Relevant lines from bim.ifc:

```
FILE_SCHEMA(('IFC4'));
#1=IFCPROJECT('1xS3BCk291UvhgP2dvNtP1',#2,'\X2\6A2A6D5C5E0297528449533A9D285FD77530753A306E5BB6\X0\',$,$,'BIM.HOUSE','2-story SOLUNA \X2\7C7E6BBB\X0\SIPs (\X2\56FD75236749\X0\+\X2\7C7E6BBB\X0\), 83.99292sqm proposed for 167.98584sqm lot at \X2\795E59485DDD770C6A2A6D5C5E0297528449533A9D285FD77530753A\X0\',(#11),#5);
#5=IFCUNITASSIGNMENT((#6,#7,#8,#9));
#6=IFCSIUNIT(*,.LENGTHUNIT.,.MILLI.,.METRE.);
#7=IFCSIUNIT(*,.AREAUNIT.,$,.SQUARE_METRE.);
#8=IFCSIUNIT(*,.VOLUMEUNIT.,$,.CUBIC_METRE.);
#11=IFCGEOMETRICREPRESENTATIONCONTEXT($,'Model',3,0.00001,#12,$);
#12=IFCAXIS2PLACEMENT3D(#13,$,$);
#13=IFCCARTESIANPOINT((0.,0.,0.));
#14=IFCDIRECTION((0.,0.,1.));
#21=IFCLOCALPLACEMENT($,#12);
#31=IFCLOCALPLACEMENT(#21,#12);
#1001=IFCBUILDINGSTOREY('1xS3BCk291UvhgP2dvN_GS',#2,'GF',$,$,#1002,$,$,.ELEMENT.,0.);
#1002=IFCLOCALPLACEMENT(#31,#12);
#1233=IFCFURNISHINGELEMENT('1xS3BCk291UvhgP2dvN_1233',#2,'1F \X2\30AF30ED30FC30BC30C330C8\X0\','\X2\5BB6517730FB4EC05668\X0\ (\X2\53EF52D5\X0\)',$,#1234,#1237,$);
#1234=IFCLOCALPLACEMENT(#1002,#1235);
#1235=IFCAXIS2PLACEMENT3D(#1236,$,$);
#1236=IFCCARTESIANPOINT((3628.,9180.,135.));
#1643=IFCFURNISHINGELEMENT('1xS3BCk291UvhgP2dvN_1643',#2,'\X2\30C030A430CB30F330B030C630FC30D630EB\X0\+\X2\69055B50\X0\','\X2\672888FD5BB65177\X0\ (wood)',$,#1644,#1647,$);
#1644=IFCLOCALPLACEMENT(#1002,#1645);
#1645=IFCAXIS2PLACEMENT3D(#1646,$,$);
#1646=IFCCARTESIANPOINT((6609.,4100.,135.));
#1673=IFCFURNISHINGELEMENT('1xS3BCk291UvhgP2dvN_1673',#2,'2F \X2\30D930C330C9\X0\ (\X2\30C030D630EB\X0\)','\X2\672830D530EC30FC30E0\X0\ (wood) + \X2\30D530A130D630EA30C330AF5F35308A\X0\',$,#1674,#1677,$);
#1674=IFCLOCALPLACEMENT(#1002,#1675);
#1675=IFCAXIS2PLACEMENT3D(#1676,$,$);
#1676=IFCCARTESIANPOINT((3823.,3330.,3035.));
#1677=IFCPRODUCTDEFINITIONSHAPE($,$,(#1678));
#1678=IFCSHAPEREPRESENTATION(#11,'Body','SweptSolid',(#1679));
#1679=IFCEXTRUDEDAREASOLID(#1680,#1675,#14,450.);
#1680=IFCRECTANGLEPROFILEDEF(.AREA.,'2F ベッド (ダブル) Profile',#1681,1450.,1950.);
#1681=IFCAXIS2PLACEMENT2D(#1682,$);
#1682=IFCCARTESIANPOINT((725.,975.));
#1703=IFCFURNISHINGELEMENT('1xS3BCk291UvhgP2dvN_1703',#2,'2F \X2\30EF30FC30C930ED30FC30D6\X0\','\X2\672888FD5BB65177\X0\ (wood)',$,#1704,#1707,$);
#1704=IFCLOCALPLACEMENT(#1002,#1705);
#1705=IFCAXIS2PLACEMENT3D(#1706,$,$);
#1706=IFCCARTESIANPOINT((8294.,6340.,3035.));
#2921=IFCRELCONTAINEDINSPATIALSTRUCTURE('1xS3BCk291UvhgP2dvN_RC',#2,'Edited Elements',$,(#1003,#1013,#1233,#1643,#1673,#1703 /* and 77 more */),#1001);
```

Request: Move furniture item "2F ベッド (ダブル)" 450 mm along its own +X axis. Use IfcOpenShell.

```python
import ifcopenshell
import ifcopenshell.api.geometry
import ifcopenshell.util.placement
import ifcopenshell.util.unit

model = ifcopenshell.open("bim.ifc")
unit_scale = ifcopenshell.util.unit.calculate_unit_scale(model)

item = model.by_id(1673)
matrix = ifcopenshell.util.placement.get_local_placement(item.ObjectPlacement)
matrix[:3, 3] += matrix[:3, 0] * 0.45 / unit_scale
ifcopenshell.api.geometry.edit_object_placement(model, product=item, matrix=matrix, is_si=False)

print(ifcopenshell.util.placement.get_local_placement(item.ObjectPlacement).round(3) + 0.0)

model.write("bim-out.ifc")
```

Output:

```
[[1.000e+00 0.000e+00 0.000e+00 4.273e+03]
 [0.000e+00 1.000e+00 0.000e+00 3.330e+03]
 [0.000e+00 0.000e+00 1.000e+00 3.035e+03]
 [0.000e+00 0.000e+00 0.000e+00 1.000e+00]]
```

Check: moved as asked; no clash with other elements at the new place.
